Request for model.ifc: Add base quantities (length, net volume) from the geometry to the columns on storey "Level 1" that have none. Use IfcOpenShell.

First a look at what the model holds.

```python
import ifcopenshell
import ifcopenshell.util.element
import ifcopenshell.util.unit

model = ifcopenshell.open("model.ifc")
print(model.schema)
for unit_type in ("LENGTHUNIT", "AREAUNIT", "VOLUMEUNIT"):
    print(unit_type, ifcopenshell.util.unit.calculate_unit_scale(model, unit_type))
storey = next(s for s in model.by_type("IfcBuildingStorey") if s.Name == "Level 1")
columns = [e for e in ifcopenshell.util.element.get_decomposition(storey) if e.is_a("IfcColumn")]
for e in sorted(columns, key=lambda e: e.id()):
    print(e.id(), e.is_a(), e.Name, list(ifcopenshell.util.element.get_psets(e, qtos_only=True)), sep=" | ")
```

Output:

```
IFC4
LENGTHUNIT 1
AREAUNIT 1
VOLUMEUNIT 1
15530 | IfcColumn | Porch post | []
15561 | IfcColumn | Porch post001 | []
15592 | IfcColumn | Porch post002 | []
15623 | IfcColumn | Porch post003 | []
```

```python
import ifcopenshell
import ifcopenshell.api.pset
import ifcopenshell.geom
import ifcopenshell.util.element
import ifcopenshell.util.shape
import ifcopenshell.util.unit

model = ifcopenshell.open("model.ifc")
unit_scale = ifcopenshell.util.unit.calculate_unit_scale(model)
volume_scale = ifcopenshell.util.unit.calculate_unit_scale(model, "VOLUMEUNIT")
settings = ifcopenshell.geom.settings()

storey = next(s for s in model.by_type("IfcBuildingStorey") if s.Name == "Level 1")
columns = [e for e in ifcopenshell.util.element.get_decomposition(storey) if e.is_a("IfcColumn")]

for e in sorted(columns, key=lambda e: e.id()):
    if ifcopenshell.util.element.get_psets(e, qtos_only=True, should_inherit=False):
        continue
    # Geometry comes back in metres, in the element's own axes.
    shape = ifcopenshell.geom.create_shape(settings, e)
    values = {
        "Length": ifcopenshell.util.shape.get_z(shape.geometry) / unit_scale,
        "NetVolume": ifcopenshell.util.shape.get_volume(shape.geometry) / volume_scale,
    }
    qto = ifcopenshell.api.pset.add_qto(model, product=e, name="Qto_ColumnBaseQuantities")
    ifcopenshell.api.pset.edit_qto(model, qto=qto, properties=values)
    print(e.id(), {k: round(v, 3) for k, v in values.items()})

model.write("model_rev.ifc")
```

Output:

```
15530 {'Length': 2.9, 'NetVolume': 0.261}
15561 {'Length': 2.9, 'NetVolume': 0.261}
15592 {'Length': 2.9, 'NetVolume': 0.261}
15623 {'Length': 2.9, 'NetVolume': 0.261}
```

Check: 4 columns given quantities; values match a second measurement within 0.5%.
